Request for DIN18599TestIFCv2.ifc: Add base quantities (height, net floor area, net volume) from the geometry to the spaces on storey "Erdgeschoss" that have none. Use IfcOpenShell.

First a look at what the model holds.

```python
import ifcopenshell
import ifcopenshell.util.element
import ifcopenshell.util.unit

model = ifcopenshell.open("DIN18599TestIFCv2.ifc")
print(model.schema)
for unit_type in ("LENGTHUNIT", "AREAUNIT", "VOLUMEUNIT"):
    print(unit_type, ifcopenshell.util.unit.calculate_unit_scale(model, unit_type))
storey = next(s for s in model.by_type("IfcBuildingStorey") if s.Name == "Erdgeschoss")
spaces = [e for e in ifcopenshell.util.element.get_decomposition(storey) if e.is_a("IfcSpace")]
for e in sorted(spaces, key=lambda e: e.id()):
    print(e.id(), e.is_a(), e.Name, list(ifcopenshell.util.element.get_psets(e, qtos_only=True)), sep=" | ")
```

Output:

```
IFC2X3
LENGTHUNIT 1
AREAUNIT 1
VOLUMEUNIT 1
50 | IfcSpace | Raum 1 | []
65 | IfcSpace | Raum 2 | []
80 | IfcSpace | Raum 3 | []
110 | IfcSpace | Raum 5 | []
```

```python
import ifcopenshell
import ifcopenshell.api.pset
import ifcopenshell.geom
import ifcopenshell.util.element
import ifcopenshell.util.shape
import ifcopenshell.util.unit

model = ifcopenshell.open("DIN18599TestIFCv2.ifc")
unit_scale = ifcopenshell.util.unit.calculate_unit_scale(model)
area_scale = ifcopenshell.util.unit.calculate_unit_scale(model, "AREAUNIT")
volume_scale = ifcopenshell.util.unit.calculate_unit_scale(model, "VOLUMEUNIT")
settings = ifcopenshell.geom.settings()

storey = next(s for s in model.by_type("IfcBuildingStorey") if s.Name == "Erdgeschoss")
spaces = [e for e in ifcopenshell.util.element.get_decomposition(storey) if e.is_a("IfcSpace")]

for e in sorted(spaces, key=lambda e: e.id()):
    if ifcopenshell.util.element.get_psets(e, qtos_only=True, should_inherit=False):
        continue
    # Geometry comes back in metres, in the element's own axes.
    shape = ifcopenshell.geom.create_shape(settings, e)
    values = {
        "Height": ifcopenshell.util.shape.get_z(shape.geometry) / unit_scale,
        "NetFloorArea": ifcopenshell.util.shape.get_footprint_area(shape.geometry) / area_scale,
        "NetVolume": ifcopenshell.util.shape.get_volume(shape.geometry) / volume_scale,
    }
    qto = ifcopenshell.api.pset.add_qto(model, product=e, name="BaseQuantities")
    ifcopenshell.api.pset.edit_qto(model, qto=qto, properties=values)
    print(e.id(), {k: round(v, 3) for k, v in values.items()})

model.write("DIN18599TestIFCv2_edited.ifc")
```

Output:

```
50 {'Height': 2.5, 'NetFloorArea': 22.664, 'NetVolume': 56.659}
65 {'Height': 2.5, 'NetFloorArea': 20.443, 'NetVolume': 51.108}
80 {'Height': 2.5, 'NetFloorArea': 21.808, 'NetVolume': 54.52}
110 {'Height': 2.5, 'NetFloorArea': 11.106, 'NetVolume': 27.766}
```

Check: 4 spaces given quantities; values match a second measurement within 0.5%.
